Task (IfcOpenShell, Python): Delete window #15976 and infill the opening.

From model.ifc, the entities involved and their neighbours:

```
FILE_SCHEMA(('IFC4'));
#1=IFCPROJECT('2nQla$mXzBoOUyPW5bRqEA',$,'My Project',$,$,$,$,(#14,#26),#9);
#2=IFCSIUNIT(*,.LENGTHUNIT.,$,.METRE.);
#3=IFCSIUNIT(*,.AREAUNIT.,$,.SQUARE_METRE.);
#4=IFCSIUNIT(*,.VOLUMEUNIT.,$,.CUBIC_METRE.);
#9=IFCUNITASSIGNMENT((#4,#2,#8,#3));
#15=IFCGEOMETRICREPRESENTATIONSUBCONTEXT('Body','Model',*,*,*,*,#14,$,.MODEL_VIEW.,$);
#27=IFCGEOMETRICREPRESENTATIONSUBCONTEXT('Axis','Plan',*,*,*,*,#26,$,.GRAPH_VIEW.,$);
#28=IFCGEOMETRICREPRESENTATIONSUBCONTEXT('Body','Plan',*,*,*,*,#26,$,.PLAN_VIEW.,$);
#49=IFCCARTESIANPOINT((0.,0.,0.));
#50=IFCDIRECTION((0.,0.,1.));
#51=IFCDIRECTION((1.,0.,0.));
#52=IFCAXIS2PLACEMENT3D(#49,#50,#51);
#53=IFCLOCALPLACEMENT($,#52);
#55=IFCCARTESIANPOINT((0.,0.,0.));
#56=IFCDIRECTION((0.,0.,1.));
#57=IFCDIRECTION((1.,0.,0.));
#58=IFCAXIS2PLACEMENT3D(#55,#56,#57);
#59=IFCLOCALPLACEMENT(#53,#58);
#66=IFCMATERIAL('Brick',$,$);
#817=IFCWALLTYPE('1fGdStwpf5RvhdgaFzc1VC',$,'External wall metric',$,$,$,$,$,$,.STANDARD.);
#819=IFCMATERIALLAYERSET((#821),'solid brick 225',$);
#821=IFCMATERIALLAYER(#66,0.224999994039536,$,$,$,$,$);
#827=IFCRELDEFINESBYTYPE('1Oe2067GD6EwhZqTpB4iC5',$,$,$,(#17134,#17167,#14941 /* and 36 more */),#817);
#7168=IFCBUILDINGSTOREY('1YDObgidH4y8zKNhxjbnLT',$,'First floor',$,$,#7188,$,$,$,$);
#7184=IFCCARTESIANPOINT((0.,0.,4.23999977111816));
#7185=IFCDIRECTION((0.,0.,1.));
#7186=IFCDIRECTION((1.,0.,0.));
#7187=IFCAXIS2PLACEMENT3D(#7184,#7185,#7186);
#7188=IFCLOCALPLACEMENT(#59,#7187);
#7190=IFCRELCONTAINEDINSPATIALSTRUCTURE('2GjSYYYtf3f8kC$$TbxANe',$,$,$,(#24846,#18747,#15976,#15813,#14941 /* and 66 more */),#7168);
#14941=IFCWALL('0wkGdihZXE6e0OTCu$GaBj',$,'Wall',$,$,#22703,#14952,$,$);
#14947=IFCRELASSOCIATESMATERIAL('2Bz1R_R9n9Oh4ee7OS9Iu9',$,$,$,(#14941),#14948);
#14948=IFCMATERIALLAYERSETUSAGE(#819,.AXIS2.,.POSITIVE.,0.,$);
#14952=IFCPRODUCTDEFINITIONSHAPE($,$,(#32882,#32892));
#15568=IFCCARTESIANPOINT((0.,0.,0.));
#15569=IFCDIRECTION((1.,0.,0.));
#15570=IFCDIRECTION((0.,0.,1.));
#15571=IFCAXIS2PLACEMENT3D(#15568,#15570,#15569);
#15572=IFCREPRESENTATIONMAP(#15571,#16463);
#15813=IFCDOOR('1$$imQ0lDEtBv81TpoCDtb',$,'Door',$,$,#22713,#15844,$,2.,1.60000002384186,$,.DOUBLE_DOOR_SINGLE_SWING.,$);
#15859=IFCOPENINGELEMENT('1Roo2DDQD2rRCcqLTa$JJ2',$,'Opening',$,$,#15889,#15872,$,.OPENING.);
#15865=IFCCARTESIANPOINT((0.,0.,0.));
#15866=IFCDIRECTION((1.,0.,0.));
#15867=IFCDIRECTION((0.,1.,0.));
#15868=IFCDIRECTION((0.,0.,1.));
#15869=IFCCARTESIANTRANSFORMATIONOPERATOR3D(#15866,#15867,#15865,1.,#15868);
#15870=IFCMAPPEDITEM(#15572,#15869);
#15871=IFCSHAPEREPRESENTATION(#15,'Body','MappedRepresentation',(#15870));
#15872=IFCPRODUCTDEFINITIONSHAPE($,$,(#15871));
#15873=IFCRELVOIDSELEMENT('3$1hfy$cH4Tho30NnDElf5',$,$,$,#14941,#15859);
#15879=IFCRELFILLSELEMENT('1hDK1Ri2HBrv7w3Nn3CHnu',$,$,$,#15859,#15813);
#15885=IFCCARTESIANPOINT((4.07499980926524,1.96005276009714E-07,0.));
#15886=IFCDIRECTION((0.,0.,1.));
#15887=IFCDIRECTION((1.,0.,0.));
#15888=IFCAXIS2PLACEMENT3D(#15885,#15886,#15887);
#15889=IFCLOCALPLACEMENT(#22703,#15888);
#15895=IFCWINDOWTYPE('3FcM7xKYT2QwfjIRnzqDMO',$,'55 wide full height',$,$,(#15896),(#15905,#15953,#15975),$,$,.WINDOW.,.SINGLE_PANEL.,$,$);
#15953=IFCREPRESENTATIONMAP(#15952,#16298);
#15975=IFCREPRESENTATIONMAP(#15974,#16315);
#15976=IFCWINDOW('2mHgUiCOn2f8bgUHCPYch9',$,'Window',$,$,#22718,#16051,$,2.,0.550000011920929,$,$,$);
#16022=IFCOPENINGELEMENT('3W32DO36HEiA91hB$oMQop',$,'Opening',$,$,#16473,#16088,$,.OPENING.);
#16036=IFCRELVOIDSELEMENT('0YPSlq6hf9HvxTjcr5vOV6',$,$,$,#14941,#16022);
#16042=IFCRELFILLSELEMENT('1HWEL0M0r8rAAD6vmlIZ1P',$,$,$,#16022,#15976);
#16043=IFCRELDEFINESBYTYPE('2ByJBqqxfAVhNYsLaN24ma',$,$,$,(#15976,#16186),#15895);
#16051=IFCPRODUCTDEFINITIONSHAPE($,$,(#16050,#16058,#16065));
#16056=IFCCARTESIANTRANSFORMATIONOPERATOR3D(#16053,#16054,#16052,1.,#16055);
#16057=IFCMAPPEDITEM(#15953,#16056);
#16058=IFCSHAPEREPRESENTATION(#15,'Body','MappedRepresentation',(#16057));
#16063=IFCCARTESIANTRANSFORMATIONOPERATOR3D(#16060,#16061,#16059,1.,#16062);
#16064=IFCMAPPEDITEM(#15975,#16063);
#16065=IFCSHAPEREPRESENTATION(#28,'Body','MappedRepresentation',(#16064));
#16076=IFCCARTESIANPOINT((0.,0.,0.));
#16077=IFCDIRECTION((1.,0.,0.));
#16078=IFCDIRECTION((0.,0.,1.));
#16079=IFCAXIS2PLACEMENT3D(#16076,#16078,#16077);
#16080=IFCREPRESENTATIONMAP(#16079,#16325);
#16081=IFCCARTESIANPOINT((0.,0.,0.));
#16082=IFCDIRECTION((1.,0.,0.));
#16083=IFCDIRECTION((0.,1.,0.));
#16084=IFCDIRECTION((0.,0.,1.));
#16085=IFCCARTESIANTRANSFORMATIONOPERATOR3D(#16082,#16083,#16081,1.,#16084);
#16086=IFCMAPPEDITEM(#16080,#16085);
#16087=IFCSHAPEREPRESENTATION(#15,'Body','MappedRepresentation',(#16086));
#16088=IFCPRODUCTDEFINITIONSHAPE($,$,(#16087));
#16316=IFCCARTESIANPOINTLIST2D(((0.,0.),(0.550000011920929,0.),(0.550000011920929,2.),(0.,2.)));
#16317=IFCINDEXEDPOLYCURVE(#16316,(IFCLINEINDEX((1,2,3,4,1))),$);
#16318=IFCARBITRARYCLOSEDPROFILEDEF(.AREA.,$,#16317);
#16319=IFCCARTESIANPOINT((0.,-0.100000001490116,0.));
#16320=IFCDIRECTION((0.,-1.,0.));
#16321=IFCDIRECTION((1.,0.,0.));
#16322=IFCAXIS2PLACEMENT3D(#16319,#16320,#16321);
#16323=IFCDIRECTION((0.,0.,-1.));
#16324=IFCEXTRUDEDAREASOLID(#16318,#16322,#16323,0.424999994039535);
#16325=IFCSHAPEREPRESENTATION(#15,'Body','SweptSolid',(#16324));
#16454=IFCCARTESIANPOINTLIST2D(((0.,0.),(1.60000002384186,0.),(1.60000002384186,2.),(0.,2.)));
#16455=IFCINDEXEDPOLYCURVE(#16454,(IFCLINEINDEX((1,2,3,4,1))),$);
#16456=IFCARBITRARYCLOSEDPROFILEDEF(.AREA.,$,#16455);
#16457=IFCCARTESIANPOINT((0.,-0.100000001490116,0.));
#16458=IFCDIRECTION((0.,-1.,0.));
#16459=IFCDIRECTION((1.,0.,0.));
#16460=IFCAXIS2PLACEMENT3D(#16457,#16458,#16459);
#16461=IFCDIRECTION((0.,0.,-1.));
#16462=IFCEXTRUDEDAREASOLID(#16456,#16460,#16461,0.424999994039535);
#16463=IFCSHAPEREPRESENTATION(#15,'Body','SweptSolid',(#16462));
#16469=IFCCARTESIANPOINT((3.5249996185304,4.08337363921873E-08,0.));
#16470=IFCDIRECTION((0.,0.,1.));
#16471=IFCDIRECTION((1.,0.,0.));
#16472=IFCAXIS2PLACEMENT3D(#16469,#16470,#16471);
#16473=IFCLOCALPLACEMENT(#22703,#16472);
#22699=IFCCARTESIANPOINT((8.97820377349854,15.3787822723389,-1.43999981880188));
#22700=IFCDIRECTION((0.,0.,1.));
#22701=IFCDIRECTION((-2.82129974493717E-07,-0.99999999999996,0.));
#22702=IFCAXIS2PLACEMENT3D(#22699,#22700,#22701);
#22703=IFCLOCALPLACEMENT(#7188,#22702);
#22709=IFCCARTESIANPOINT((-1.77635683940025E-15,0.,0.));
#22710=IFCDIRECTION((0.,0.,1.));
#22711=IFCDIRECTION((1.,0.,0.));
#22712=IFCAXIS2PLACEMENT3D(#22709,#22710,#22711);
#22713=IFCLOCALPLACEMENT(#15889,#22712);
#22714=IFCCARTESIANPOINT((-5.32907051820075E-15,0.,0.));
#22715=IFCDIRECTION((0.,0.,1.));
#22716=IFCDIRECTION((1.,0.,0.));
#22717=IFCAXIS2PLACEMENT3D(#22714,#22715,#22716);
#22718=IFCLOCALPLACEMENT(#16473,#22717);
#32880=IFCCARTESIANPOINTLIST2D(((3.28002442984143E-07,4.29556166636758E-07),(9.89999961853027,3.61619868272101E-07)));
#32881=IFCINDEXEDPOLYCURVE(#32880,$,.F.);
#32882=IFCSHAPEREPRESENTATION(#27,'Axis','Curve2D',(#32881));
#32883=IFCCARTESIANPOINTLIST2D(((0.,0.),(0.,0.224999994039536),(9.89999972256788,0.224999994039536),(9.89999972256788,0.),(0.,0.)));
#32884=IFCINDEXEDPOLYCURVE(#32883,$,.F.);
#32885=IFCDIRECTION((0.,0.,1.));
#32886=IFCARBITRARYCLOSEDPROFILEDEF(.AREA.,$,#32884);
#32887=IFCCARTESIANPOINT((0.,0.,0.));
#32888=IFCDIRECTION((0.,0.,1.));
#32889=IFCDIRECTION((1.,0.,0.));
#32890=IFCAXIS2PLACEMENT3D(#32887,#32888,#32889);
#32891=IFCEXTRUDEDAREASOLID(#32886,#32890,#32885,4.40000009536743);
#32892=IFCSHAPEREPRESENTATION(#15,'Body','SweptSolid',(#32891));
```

```python
import ifcopenshell
import ifcopenshell.api.feature
import ifcopenshell.api.root
import ifcopenshell.geom
import ifcopenshell.util.shape

model = ifcopenshell.open("model.ifc")
settings = ifcopenshell.geom.settings()


def volume(element):
    """Net volume in cubic metres, openings subtracted."""
    shape = ifcopenshell.geom.create_shape(settings, element)
    return ifcopenshell.util.shape.get_volume(shape.geometry)


window = model.by_id(15976)
opening = window.FillsVoids[0].RelatingOpeningElement
wall = opening.VoidsElements[0].RelatingBuildingElement
before = volume(wall)

ifcopenshell.api.root.remove_product(model, product=window)
ifcopenshell.api.feature.remove_feature(model, feature=opening)

after = volume(wall)

print(f"wall volume {before:.3f} -> {after:.3f} m3")

model.write("model-out.ifc")
```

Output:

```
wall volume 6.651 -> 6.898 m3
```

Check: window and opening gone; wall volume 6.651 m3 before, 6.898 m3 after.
